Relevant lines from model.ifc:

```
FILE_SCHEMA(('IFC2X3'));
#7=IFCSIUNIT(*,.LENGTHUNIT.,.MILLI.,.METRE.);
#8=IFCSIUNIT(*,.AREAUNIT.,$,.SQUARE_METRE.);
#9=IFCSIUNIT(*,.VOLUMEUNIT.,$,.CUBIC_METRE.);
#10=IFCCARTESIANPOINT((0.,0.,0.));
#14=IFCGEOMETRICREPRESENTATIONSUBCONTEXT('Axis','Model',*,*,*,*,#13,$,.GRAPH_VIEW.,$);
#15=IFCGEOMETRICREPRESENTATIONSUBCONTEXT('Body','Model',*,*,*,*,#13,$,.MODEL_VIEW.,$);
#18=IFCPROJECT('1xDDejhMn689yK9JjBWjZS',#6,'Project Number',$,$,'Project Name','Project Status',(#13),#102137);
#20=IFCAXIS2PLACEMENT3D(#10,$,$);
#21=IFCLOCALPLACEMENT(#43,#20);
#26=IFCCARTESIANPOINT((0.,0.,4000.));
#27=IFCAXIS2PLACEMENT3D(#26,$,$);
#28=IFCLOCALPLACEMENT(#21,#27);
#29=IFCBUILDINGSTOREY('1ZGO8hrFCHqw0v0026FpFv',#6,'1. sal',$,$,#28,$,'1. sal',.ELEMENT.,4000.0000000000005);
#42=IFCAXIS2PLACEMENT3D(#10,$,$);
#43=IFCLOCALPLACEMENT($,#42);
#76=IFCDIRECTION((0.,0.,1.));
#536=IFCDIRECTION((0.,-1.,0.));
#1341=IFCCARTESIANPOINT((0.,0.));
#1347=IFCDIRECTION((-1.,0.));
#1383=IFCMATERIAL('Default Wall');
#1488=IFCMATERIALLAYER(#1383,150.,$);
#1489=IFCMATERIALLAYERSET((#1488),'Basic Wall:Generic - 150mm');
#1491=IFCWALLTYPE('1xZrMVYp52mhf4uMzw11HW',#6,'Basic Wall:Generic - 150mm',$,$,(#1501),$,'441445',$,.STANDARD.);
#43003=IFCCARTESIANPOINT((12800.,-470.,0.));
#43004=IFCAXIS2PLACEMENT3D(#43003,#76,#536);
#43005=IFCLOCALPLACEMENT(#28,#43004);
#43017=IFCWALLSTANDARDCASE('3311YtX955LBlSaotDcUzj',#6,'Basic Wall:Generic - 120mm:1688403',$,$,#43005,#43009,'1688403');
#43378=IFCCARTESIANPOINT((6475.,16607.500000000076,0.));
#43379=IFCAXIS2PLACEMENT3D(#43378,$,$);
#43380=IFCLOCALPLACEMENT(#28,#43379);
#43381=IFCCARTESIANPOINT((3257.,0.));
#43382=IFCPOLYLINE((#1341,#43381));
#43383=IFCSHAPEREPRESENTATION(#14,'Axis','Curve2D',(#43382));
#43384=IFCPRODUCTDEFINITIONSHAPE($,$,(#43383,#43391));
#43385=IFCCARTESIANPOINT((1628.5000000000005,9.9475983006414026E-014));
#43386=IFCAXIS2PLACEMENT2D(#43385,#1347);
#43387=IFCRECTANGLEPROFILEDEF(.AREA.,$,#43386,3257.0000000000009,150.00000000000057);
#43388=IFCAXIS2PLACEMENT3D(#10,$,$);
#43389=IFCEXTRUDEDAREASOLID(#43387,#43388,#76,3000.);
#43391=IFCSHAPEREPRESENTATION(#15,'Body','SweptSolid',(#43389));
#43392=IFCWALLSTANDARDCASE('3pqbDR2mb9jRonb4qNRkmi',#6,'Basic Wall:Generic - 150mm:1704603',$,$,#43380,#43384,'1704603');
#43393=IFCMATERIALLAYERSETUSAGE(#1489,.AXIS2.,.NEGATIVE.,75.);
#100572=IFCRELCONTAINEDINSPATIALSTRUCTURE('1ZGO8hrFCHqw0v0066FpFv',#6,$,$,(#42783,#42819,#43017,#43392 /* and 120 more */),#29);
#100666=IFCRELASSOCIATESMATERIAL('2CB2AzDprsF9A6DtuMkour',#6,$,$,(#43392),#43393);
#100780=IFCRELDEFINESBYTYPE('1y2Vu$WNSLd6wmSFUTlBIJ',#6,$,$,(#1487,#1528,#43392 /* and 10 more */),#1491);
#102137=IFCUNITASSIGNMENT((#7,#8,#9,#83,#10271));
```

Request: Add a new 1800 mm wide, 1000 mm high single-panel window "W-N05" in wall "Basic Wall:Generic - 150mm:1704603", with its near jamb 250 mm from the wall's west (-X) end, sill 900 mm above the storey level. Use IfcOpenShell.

```python
import numpy as np
import ifcopenshell
import ifcopenshell.api.feature
import ifcopenshell.api.geometry
import ifcopenshell.api.root
import ifcopenshell.api.spatial
import ifcopenshell.api.type
import ifcopenshell.geom
import ifcopenshell.util.element
import ifcopenshell.util.placement
import ifcopenshell.util.representation
import ifcopenshell.util.shape
import ifcopenshell.util.unit

model = ifcopenshell.open("model.ifc")
unit_scale = ifcopenshell.util.unit.calculate_unit_scale(model)
settings = ifcopenshell.geom.settings()


def volume(element):
    """Net volume in cubic metres, openings subtracted."""
    shape = ifcopenshell.geom.create_shape(settings, element)
    return ifcopenshell.util.shape.get_volume(shape.geometry)


wall = model.by_guid("3pqbDR2mb9jRonb4qNRkmi")
storey = ifcopenshell.util.element.get_container(wall, ifc_class="IfcBuildingStorey")
context = ifcopenshell.util.representation.get_context(model, "Model", "Body", "MODEL_VIEW")
before = volume(wall)

width, height, from_end, sill = 1.8, 1, 0.25, 0.9  # metres

# The wall runs along its own X axis, and the end named is its -X end.
wall_shape = ifcopenshell.geom.create_shape(settings, wall)
x, y, z = ifcopenshell.util.shape.get_vertices(wall_shape.geometry).T
start = x.min() + from_end
face, thickness = float(y.min()), float(y.max() - y.min())
wall_matrix = ifcopenshell.util.placement.get_local_placement(wall.ObjectPlacement)
level = ifcopenshell.util.placement.get_local_placement(storey.ObjectPlacement)[2, 3]


def in_wall(x, y):
    """Placement at x, y metres in the wall's axes, at sill height."""
    matrix = wall_matrix.copy()
    matrix[:, 3] = wall_matrix @ np.array([x / unit_scale, y / unit_scale, 0.0, 1.0])
    matrix[2, 3] = level + sill / unit_scale
    return matrix


# Opening: a box that overshoots both wall faces by 50 mm.
opening = ifcopenshell.api.root.create_entity(model, ifc_class="IfcOpeningElement")
box = ifcopenshell.api.geometry.add_wall_representation(
    model, context=context, length=width, height=height, thickness=thickness + 0.1
)
ifcopenshell.api.geometry.assign_representation(model, product=opening, representation=box)
ifcopenshell.api.geometry.edit_object_placement(model, product=opening, matrix=in_wall(start, face - 0.05), is_si=False)
ifcopenshell.api.feature.add_feature(model, feature=opening, element=wall)

window = ifcopenshell.api.root.create_entity(model, ifc_class="IfcWindow", name="W-N05")
window.OverallWidth, window.OverallHeight = width / unit_scale, height / unit_scale
body = ifcopenshell.api.geometry.add_window_representation(
    model,
    context=context,
    overall_width=window.OverallWidth,
    overall_height=window.OverallHeight,
    partition_type="SINGLE_PANEL",
)
ifcopenshell.api.geometry.assign_representation(model, product=window, representation=body)
ifcopenshell.api.spatial.assign_container(model, products=[window], relating_structure=storey)
fills = ifcopenshell.api.feature.add_filling(model, opening=opening, element=window)
fills.OwnerHistory = window.OwnerHistory  # required in IFC2X3

# IFC2X3 keeps the operation on the window style.
style = ifcopenshell.api.root.create_entity(model, ifc_class="IfcWindowStyle", name="W-N05")
style.OperationType, style.ConstructionType = "SINGLE_PANEL", "NOTDEFINED"
style.ParameterTakesPrecedence = style.Sizeable = False
ifcopenshell.api.type.assign_type(model, related_objects=[window], relating_type=style)

# Centre the window in the wall's thickness.
ifcopenshell.api.geometry.edit_object_placement(model, product=window, matrix=in_wall(start, face), is_si=False)
window_shape = ifcopenshell.geom.create_shape(settings, window)
depth = ifcopenshell.util.shape.get_vertices(window_shape.geometry)[:, 1]
offset = face + thickness / 2 - (depth.min() + depth.max()) / 2
ifcopenshell.api.geometry.edit_object_placement(model, product=window, matrix=in_wall(start, offset), is_si=False)

after = volume(wall)

print(f"wall volume {before:.3f} -> {after:.3f} m3")

model.write("model-out.ifc")
```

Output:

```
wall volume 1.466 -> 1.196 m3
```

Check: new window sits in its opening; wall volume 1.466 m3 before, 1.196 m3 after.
